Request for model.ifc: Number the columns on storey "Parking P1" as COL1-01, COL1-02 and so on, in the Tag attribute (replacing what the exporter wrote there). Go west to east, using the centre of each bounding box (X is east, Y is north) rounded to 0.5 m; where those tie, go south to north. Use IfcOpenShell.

First a look at what the model holds.

```python
import ifcopenshell
import ifcopenshell.util.element
import ifcopenshell.util.placement

model = ifcopenshell.open("model.ifc")
print(model.schema)
storey = next(s for s in model.by_type("IfcBuildingStorey") if s.Name == "Parking P1")
columns = [e for e in ifcopenshell.util.element.get_decomposition(storey) if e.is_a("IfcColumn")]
for e in sorted(columns, key=lambda e: e.id()):
    origin = ifcopenshell.util.placement.get_local_placement(e.ObjectPlacement)[:3, 3]
    print(e.id(), e.Tag, e.Name, origin.round(2) + 0.0, sep=" | ")
```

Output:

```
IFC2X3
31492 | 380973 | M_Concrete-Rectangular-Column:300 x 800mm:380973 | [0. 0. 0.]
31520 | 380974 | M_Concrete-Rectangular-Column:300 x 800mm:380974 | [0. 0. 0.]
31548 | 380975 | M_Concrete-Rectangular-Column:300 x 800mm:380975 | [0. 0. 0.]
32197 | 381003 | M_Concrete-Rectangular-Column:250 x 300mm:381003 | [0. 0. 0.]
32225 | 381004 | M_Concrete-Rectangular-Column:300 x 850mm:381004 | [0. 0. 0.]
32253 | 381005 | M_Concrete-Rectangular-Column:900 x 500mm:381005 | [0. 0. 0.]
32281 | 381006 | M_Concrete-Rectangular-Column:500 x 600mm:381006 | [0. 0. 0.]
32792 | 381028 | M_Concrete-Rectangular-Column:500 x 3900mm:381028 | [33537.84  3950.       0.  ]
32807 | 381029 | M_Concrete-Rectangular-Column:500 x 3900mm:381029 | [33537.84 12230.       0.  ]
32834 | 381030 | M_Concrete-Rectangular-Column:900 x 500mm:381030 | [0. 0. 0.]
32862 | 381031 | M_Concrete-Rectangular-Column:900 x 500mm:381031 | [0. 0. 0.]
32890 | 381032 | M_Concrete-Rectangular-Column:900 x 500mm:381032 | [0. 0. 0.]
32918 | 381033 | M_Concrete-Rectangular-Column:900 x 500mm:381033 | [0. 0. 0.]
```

```python
import ifcopenshell
import ifcopenshell.geom
import ifcopenshell.util.element
import ifcopenshell.util.shape

model = ifcopenshell.open("model.ifc")
settings = ifcopenshell.geom.settings()
settings.set("use-world-coords", True)


def centre(element):
    shape = ifcopenshell.geom.create_shape(settings, element)
    return ifcopenshell.util.shape.get_bbox_centroid(shape.geometry)


storey = next(s for s in model.by_type("IfcBuildingStorey") if s.Name == "Parking P1")
columns = [e for e in ifcopenshell.util.element.get_decomposition(storey) if e.is_a("IfcColumn")]

# Insertion points can sit at a corner or the storey origin, so sort by the geometry (in metres).
centres = {e: centre(e) for e in columns}
columns.sort(key=lambda e: (round(centres[e][0] / 0.5), centres[e][1]))

for i, e in enumerate(columns, start=1):
    number = f"COL1-{i:02d}"
    e.Tag = number
    print(e.id(), number)

model.write("model_edited.ifc")
```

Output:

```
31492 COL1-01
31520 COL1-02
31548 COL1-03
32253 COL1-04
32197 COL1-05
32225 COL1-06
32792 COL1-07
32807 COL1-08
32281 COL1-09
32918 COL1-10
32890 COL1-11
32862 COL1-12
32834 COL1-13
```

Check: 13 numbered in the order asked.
